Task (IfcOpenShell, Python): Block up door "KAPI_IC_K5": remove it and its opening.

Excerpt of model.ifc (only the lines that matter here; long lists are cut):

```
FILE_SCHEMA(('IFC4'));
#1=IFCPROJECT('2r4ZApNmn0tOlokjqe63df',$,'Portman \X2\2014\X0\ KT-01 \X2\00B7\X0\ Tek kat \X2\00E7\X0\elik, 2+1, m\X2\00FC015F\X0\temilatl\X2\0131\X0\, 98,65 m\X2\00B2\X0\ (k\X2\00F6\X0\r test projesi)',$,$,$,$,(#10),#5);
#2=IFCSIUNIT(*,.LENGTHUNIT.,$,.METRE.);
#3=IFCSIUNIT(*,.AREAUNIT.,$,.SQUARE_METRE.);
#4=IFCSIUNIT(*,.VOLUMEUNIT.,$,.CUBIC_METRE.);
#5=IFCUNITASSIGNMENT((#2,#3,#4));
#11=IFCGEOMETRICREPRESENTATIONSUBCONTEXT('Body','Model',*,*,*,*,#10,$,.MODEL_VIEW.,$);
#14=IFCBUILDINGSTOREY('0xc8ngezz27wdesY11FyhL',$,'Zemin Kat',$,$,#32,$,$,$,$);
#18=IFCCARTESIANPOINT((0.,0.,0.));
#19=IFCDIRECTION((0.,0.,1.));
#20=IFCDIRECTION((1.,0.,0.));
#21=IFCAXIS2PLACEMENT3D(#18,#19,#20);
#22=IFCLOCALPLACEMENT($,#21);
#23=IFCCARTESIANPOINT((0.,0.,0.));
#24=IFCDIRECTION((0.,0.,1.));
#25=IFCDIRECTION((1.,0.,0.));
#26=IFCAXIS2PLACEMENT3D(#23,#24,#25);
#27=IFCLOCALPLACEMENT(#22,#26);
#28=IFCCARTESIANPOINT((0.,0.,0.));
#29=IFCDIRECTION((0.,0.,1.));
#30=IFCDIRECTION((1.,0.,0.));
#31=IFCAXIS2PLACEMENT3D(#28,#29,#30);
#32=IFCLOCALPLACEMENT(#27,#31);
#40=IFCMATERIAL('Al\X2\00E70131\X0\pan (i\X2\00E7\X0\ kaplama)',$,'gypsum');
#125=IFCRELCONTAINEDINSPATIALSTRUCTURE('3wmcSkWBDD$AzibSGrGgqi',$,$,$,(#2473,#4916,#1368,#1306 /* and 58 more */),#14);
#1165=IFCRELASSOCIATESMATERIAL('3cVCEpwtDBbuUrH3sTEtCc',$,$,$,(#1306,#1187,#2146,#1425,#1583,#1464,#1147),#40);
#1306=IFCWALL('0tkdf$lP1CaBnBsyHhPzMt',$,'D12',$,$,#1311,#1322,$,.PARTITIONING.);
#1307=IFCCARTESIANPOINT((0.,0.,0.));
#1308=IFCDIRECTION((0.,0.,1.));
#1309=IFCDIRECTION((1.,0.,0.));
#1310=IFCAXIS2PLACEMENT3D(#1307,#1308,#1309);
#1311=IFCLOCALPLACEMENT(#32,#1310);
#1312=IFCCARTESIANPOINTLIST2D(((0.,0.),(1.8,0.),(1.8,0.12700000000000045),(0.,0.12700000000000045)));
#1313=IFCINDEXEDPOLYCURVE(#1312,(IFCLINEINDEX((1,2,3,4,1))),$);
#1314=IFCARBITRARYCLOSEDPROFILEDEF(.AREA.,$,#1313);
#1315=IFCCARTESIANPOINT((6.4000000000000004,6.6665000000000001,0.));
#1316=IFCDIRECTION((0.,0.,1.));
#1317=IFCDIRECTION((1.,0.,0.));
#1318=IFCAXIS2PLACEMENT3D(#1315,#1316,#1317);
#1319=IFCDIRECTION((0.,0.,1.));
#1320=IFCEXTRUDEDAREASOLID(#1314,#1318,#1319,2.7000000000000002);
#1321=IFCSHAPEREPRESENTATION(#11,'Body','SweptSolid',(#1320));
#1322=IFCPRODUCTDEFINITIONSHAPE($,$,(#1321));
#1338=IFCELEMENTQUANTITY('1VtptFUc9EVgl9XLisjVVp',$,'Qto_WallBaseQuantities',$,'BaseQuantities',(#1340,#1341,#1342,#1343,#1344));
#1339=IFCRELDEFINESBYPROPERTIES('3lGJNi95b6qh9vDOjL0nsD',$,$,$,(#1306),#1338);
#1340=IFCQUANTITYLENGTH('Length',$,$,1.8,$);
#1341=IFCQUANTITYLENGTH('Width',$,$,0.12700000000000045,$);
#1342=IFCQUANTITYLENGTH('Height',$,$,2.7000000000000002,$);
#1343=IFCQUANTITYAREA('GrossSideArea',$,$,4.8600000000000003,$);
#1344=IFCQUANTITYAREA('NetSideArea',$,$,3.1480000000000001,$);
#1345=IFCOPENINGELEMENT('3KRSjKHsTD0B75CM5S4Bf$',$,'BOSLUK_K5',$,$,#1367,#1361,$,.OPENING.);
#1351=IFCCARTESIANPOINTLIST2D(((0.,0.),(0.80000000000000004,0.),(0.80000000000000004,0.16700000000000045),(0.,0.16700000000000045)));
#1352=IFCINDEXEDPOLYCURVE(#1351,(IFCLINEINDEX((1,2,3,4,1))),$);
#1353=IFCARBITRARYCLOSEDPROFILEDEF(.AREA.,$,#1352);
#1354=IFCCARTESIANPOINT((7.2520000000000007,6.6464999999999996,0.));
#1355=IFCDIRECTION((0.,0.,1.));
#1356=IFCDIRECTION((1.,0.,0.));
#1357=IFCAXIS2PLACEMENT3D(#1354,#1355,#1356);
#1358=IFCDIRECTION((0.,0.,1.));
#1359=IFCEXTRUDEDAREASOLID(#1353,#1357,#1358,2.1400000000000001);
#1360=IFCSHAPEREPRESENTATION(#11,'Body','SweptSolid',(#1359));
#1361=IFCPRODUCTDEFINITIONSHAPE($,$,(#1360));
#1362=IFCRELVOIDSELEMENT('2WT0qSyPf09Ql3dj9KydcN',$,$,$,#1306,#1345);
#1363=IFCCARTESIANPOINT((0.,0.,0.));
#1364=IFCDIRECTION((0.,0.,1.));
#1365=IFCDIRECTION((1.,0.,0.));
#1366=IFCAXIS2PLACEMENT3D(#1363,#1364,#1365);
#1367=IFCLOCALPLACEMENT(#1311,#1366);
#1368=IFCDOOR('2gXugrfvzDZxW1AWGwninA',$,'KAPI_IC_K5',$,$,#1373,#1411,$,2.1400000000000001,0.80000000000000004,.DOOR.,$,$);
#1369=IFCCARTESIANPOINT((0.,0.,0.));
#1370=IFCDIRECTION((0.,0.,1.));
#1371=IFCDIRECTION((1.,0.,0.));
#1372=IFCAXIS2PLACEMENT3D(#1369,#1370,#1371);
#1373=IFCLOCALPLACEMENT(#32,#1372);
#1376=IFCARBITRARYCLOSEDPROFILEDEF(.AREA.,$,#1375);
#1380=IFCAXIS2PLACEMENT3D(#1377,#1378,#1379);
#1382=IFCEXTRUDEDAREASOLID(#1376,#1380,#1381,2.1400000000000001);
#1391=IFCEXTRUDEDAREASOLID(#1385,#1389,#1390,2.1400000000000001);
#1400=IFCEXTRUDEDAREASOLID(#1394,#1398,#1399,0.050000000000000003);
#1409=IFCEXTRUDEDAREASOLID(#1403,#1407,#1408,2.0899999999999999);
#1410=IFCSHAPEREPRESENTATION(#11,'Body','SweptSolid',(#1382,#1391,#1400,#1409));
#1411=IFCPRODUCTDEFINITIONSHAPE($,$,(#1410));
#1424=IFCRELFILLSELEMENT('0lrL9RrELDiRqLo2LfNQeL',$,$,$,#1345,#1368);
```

```python
import ifcopenshell
import ifcopenshell.api.feature
import ifcopenshell.api.pset
import ifcopenshell.api.root
import ifcopenshell.geom
import ifcopenshell.util.element
import ifcopenshell.util.shape
import ifcopenshell.util.unit

model = ifcopenshell.open("model.ifc")
area_scale = ifcopenshell.util.unit.calculate_unit_scale(model, "AREAUNIT")
settings = ifcopenshell.geom.settings()


def volume(element):
    """Net volume in cubic metres, openings subtracted."""
    shape = ifcopenshell.geom.create_shape(settings, element)
    return ifcopenshell.util.shape.get_volume(shape.geometry)


door = model.by_guid("2gXugrfvzDZxW1AWGwninA")
opening = door.FillsVoids[0].RelatingOpeningElement
wall = opening.VoidsElements[0].RelatingBuildingElement
before = volume(wall)

ifcopenshell.api.root.remove_product(model, product=door)
ifcopenshell.api.feature.remove_feature(model, feature=opening)

after = volume(wall)
thickness = 0.127  # wall thickness in metres

# Update the wall's stored quantities.
qto = model.by_id(ifcopenshell.util.element.get_pset(wall, "Qto_WallBaseQuantities", should_inherit=False)["id"])
ifcopenshell.api.pset.edit_qto(model, qto=qto, properties={"NetSideArea": after / thickness / area_scale})

print(f"wall volume {before:.3f} -> {after:.3f} m3")

model.write("model_v2.ifc")
```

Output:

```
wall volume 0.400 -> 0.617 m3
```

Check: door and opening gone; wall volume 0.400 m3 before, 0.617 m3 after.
